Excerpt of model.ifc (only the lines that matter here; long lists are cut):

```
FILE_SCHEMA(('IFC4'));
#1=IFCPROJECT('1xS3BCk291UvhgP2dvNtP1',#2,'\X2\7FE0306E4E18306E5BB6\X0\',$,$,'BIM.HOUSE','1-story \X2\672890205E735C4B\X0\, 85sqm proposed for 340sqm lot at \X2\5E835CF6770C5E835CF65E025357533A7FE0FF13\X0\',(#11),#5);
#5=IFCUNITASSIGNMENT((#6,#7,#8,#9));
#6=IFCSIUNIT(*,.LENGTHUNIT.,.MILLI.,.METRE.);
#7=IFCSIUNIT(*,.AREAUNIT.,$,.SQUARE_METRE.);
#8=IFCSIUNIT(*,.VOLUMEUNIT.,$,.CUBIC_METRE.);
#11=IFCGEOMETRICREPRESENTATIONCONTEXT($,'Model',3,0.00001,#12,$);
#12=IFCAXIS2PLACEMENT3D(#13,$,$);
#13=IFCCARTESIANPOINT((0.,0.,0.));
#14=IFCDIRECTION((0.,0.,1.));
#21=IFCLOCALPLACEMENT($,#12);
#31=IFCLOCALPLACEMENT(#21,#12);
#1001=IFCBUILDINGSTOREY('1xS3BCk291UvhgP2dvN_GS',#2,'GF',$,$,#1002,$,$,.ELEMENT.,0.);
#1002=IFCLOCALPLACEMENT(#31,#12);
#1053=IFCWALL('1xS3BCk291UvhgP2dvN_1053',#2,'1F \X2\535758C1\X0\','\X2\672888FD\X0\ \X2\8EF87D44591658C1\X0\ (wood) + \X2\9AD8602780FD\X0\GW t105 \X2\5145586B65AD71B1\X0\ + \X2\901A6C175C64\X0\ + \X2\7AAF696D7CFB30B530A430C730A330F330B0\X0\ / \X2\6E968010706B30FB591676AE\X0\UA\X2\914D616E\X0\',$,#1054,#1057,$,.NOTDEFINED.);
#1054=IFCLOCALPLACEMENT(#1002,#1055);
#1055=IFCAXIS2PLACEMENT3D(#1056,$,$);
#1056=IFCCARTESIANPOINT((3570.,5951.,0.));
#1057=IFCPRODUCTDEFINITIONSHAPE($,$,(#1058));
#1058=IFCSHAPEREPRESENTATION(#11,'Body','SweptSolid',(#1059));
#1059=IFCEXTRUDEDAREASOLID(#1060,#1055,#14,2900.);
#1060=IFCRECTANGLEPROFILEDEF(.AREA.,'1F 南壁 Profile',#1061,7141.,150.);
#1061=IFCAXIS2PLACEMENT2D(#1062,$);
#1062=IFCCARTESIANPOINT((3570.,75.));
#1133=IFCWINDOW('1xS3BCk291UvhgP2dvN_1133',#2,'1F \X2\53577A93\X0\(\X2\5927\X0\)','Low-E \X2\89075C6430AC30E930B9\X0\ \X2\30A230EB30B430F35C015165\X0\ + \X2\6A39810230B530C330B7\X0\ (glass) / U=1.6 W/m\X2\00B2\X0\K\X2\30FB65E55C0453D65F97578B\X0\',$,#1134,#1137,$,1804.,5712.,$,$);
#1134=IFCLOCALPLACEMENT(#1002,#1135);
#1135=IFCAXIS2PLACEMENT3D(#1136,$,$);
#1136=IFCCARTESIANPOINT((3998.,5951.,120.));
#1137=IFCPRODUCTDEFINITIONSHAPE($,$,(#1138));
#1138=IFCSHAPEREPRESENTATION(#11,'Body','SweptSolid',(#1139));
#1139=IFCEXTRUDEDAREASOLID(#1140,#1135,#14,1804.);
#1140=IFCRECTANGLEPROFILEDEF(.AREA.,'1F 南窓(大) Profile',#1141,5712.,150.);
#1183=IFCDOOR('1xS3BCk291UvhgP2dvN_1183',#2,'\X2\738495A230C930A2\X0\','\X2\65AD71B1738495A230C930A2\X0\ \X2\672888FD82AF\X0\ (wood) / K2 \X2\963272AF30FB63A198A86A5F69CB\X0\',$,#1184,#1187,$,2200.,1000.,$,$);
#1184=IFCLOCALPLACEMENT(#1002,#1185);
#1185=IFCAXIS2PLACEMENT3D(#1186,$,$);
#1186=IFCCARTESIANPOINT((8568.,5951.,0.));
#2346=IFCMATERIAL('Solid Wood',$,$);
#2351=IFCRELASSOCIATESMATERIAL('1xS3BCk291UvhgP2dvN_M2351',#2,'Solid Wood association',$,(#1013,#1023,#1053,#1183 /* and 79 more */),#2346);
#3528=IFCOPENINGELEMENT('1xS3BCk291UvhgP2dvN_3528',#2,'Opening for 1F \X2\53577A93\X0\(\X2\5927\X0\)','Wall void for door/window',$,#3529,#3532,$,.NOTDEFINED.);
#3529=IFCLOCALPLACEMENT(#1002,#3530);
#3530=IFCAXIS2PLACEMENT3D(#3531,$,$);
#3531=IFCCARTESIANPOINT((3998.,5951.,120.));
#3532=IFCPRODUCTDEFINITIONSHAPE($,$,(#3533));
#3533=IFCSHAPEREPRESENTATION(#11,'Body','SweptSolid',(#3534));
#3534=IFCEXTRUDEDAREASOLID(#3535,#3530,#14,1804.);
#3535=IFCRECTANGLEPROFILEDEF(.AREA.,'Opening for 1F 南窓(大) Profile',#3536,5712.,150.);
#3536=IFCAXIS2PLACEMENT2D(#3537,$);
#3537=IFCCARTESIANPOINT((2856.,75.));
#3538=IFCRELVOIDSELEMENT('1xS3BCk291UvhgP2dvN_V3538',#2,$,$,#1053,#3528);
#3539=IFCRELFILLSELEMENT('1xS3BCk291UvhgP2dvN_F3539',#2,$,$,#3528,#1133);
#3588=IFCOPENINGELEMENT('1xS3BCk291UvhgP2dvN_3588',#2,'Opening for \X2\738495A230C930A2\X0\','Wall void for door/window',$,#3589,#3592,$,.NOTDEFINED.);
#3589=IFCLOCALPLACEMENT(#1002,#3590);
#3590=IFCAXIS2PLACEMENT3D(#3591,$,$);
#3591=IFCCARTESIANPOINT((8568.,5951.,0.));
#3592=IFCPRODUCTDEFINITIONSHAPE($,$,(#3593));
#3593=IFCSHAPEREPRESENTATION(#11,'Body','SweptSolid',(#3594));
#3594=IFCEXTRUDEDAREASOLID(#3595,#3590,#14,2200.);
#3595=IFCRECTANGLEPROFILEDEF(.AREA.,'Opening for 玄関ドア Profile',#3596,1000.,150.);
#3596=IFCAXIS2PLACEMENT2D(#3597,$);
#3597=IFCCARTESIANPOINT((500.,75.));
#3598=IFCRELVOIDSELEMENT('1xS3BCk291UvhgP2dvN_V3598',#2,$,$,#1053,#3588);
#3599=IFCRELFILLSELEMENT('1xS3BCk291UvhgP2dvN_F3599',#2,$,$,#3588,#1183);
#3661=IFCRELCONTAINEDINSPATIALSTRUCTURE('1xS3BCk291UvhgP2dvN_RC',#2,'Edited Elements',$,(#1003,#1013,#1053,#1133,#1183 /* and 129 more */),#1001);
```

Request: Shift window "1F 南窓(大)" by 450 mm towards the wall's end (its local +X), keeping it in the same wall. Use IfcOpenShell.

```python
import ifcopenshell
import ifcopenshell.api.geometry
import ifcopenshell.util.placement
import ifcopenshell.util.unit

model = ifcopenshell.open("model.ifc")
unit_scale = ifcopenshell.util.unit.calculate_unit_scale(model)

window = model.by_guid("1xS3BCk291UvhgP2dvN_1133")
opening = window.FillsVoids[0].RelatingOpeningElement
wall = opening.VoidsElements[0].RelatingBuildingElement

wall_matrix = ifcopenshell.util.placement.get_local_placement(wall.ObjectPlacement)
shift = wall_matrix[:3, 0] * 0.45 / unit_scale
before = ifcopenshell.util.placement.get_local_placement(window.ObjectPlacement)[:3, 3].copy()

# The window is not placed relative to its opening, so move both.
for product in (opening, window):
    matrix = ifcopenshell.util.placement.get_local_placement(product.ObjectPlacement)
    matrix[:3, 3] += shift
    ifcopenshell.api.geometry.edit_object_placement(model, product=product, matrix=matrix, is_si=False)

after = ifcopenshell.util.placement.get_local_placement(window.ObjectPlacement)[:3, 3]
print("window moved by", (after - before).round(3) + 0.0)

model.write("model_edited.ifc")
```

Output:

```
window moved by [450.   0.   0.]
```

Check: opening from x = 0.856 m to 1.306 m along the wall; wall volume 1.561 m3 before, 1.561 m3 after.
